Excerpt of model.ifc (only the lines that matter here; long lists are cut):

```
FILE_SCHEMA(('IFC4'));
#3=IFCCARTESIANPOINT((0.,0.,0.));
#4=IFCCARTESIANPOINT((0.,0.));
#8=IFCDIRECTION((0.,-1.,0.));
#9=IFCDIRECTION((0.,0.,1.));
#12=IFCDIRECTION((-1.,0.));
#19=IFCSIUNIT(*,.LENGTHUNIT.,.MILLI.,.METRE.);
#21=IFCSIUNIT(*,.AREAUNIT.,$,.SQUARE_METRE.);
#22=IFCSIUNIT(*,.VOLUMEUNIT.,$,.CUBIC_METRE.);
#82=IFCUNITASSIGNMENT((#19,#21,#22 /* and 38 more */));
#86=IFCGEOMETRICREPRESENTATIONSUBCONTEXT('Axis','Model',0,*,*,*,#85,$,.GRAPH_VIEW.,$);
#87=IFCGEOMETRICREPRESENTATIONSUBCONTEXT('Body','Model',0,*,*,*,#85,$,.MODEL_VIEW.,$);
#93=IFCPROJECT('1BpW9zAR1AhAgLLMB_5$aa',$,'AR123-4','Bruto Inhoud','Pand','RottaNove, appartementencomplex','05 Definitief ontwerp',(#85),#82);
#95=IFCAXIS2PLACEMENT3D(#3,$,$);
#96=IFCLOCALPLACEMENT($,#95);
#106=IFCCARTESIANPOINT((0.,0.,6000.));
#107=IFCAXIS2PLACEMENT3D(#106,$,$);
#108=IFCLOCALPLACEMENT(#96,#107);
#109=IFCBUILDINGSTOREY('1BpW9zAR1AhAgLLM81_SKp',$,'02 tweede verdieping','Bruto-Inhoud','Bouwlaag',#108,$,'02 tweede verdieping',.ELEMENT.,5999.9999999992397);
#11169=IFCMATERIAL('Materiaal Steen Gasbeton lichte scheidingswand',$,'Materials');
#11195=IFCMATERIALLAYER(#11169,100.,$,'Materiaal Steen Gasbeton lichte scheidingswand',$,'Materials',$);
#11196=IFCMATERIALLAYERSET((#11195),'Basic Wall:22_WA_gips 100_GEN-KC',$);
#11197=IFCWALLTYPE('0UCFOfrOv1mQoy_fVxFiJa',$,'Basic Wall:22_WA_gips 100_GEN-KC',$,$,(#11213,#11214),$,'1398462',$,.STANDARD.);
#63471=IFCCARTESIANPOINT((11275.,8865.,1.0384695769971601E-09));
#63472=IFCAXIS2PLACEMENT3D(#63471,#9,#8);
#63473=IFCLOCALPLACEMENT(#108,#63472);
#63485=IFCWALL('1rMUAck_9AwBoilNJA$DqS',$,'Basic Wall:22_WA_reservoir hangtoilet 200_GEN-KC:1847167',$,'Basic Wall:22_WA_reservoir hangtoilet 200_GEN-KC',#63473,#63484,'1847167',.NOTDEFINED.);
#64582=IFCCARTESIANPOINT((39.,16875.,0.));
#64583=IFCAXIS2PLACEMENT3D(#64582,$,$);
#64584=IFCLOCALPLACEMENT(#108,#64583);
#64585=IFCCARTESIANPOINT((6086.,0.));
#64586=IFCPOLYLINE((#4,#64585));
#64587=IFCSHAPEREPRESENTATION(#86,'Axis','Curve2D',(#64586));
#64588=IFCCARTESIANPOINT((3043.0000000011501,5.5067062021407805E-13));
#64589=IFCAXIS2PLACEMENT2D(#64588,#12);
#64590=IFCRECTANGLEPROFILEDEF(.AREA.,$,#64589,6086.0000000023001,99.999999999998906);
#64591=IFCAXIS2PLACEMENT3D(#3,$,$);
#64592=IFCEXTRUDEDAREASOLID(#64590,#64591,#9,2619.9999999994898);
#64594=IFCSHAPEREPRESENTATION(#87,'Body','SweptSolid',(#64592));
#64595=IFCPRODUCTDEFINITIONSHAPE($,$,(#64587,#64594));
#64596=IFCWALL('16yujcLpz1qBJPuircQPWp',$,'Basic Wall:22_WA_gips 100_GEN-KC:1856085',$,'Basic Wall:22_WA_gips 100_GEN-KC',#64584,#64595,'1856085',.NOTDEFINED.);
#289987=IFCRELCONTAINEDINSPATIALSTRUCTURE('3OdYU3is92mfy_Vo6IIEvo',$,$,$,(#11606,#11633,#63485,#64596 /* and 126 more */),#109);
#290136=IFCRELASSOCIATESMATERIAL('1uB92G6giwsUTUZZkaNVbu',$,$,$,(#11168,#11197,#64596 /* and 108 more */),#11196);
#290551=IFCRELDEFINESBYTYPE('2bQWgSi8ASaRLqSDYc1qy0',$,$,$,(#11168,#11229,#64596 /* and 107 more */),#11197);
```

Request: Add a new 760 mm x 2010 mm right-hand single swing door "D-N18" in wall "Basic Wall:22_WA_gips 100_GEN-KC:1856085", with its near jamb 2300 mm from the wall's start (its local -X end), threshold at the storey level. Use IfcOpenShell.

```python
import numpy as np
import ifcopenshell
import ifcopenshell.api.feature
import ifcopenshell.api.geometry
import ifcopenshell.api.root
import ifcopenshell.api.spatial
import ifcopenshell.geom
import ifcopenshell.util.element
import ifcopenshell.util.placement
import ifcopenshell.util.representation
import ifcopenshell.util.shape
import ifcopenshell.util.unit

model = ifcopenshell.open("model.ifc")
unit_scale = ifcopenshell.util.unit.calculate_unit_scale(model)
settings = ifcopenshell.geom.settings()


def volume(element):
    """Net volume in cubic metres, openings subtracted."""
    shape = ifcopenshell.geom.create_shape(settings, element)
    return ifcopenshell.util.shape.get_volume(shape.geometry)


wall = model.by_guid("16yujcLpz1qBJPuircQPWp")
storey = ifcopenshell.util.element.get_container(wall, ifc_class="IfcBuildingStorey")
context = ifcopenshell.util.representation.get_context(model, "Model", "Body", "MODEL_VIEW")
before = volume(wall)

width, height, from_end, sill = 0.76, 2.01, 2.3, 0.0  # metres

# The wall runs along its own X axis, and the end named is its -X end.
wall_shape = ifcopenshell.geom.create_shape(settings, wall)
x, y, z = ifcopenshell.util.shape.get_vertices(wall_shape.geometry).T
start = x.min() + from_end
face, thickness = float(y.min()), float(y.max() - y.min())
wall_matrix = ifcopenshell.util.placement.get_local_placement(wall.ObjectPlacement)
level = ifcopenshell.util.placement.get_local_placement(storey.ObjectPlacement)[2, 3]


def in_wall(x, y):
    """Placement at x, y metres in the wall's axes, at sill height."""
    matrix = wall_matrix.copy()
    matrix[:, 3] = wall_matrix @ np.array([x / unit_scale, y / unit_scale, 0.0, 1.0])
    matrix[2, 3] = level + sill / unit_scale
    return matrix


# Opening: a box that overshoots both wall faces by 50 mm.
opening = ifcopenshell.api.root.create_entity(model, ifc_class="IfcOpeningElement", predefined_type="OPENING")
box = ifcopenshell.api.geometry.add_wall_representation(
    model, context=context, length=width, height=height, thickness=thickness + 0.1
)
ifcopenshell.api.geometry.assign_representation(model, product=opening, representation=box)
ifcopenshell.api.geometry.edit_object_placement(model, product=opening, matrix=in_wall(start, face - 0.05), is_si=False)
ifcopenshell.api.feature.add_feature(model, feature=opening, element=wall)

door = ifcopenshell.api.root.create_entity(model, ifc_class="IfcDoor", name="D-N18", predefined_type="DOOR")
door.OverallWidth, door.OverallHeight = width / unit_scale, height / unit_scale
door.OperationType = "SINGLE_SWING_RIGHT"
body = ifcopenshell.api.geometry.add_door_representation(
    model,
    context=context,
    overall_width=door.OverallWidth,
    overall_height=door.OverallHeight,
    operation_type="SINGLE_SWING_RIGHT",
    lining_properties={"LiningDepth": thickness / unit_scale, "ThresholdDepth": thickness / unit_scale},
)
ifcopenshell.api.geometry.assign_representation(model, product=door, representation=body)
ifcopenshell.api.spatial.assign_container(model, products=[door], relating_structure=storey)
ifcopenshell.api.feature.add_filling(model, opening=opening, element=door)

# The lining spans the wall, so the door starts at the wall face.
ifcopenshell.api.geometry.edit_object_placement(model, product=door, matrix=in_wall(start, face), is_si=False)

after = volume(wall)

print(f"wall volume {before:.3f} -> {after:.3f} m3")

model.write("model_updated.ifc")
```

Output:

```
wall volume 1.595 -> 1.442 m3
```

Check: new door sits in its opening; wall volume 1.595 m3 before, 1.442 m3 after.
